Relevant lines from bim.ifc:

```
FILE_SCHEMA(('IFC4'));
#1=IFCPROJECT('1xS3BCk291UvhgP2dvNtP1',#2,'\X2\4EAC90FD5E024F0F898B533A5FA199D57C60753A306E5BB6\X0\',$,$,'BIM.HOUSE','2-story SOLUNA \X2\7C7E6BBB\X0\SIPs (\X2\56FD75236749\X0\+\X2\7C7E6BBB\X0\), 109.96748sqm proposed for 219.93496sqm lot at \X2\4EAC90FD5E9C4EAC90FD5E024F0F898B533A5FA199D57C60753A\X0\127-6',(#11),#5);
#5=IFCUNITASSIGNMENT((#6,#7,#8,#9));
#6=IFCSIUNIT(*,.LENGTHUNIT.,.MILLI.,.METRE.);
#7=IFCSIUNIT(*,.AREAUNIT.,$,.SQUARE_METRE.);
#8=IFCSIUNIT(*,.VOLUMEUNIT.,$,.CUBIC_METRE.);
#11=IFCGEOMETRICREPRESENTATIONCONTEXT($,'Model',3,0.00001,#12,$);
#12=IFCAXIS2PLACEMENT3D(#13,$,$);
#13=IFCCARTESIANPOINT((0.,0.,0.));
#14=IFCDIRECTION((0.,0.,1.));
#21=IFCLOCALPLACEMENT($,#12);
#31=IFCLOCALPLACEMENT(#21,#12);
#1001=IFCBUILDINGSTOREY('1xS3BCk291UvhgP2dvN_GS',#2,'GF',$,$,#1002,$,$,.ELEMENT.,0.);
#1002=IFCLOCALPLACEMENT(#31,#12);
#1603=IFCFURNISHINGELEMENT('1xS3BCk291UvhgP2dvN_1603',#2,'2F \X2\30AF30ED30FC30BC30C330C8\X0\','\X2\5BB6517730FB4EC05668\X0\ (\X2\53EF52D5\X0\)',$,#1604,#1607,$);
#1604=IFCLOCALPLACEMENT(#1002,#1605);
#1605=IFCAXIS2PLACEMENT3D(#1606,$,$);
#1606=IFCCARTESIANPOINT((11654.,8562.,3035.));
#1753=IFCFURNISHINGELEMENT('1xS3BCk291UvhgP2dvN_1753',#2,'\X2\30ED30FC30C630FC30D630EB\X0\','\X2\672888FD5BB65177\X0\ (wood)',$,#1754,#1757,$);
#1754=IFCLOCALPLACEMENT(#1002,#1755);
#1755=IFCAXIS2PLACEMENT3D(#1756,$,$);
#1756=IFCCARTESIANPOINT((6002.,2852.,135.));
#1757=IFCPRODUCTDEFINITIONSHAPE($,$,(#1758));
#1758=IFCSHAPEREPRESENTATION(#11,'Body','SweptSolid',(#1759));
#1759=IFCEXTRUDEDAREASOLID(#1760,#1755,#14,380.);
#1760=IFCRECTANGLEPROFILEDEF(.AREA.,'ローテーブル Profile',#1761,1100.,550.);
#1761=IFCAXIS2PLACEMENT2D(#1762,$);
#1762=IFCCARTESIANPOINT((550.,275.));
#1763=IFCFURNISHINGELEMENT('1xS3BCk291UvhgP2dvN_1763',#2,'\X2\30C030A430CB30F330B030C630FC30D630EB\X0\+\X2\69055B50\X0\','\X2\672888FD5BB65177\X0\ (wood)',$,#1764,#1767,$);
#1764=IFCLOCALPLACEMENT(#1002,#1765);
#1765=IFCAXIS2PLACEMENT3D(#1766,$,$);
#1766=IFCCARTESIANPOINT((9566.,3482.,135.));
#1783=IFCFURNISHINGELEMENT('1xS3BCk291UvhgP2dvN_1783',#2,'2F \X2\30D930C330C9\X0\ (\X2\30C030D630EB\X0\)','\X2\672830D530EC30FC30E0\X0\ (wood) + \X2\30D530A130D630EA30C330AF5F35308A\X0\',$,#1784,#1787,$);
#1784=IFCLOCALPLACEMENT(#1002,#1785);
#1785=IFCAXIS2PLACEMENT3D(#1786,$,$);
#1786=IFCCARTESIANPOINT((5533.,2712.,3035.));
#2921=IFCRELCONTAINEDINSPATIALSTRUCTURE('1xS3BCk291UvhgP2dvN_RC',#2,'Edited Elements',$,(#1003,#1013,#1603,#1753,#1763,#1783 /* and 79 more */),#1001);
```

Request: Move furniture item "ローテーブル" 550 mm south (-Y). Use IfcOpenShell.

```python
import ifcopenshell
import ifcopenshell.api.geometry
import ifcopenshell.util.placement

model = ifcopenshell.open("bim.ifc")

item = model.by_id(1753)
matrix = ifcopenshell.util.placement.get_local_placement(item.ObjectPlacement)
matrix[1, 3] -= 550.0
ifcopenshell.api.geometry.edit_object_placement(model, product=item, matrix=matrix, is_si=False)

print(ifcopenshell.util.placement.get_local_placement(item.ObjectPlacement).round(3) + 0.0)

model.write("bim_updated.ifc")
```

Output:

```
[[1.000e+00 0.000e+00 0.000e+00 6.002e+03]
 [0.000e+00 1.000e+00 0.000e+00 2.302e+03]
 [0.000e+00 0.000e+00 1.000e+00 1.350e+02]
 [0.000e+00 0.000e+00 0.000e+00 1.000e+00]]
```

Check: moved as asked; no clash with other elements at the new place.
